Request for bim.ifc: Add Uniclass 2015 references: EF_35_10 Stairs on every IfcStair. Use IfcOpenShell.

First a look at what the model holds.

```python
import ifcopenshell

model = ifcopenshell.open("bim.ifc")
print(model.schema)
print("classifications:", [c.Name for c in model.by_type("IfcClassification")])
for ifc_class in ("IfcDoor", "IfcRoof", "IfcStair", "IfcWall", "IfcWindow"):
    print(ifc_class, len(model.by_type(ifc_class)))
```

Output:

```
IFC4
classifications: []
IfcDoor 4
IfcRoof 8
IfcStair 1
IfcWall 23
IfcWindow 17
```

```python
import ifcopenshell
import ifcopenshell.api.classification

model = ifcopenshell.open("bim.ifc")

system = ifcopenshell.api.classification.add_classification(model, classification="Uniclass 2015")

codes = {
    "IfcStair": ("EF_35_10", "Stairs"),
}
for ifc_class, (code, name) in codes.items():
    products = model.by_type(ifc_class)
    ifcopenshell.api.classification.add_reference(
        model, products=products, classification=system, identification=code, name=name
    )
    print(code, len(products))

model.write("bim_updated.ifc")
```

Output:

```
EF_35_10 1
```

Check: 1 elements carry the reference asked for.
